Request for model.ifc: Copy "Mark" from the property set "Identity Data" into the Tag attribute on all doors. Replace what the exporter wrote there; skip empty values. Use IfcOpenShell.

First a look at what the model holds.

```python
import ifcopenshell
import ifcopenshell.util.element

model = ifcopenshell.open("model.ifc")
print(model.schema)
doors = model.by_type("IfcDoor")
print(len(doors), "doors")
for e in doors[:8]:
    source = ifcopenshell.util.element.get_pset(e, "Identity Data", "Mark")
    target = e.Tag
    print(e.id(), repr(source), repr(target), sep=" | ")
```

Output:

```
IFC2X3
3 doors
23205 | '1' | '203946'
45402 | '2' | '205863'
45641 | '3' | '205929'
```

```python
import ifcopenshell
import ifcopenshell.util.element

model = ifcopenshell.open("model.ifc")

count = 0
for e in model.by_type("IfcDoor"):
    value = ifcopenshell.util.element.get_pset(e, "Identity Data", "Mark")
    current = e.Tag
    if not value or not value.strip() or current == value:
        continue
    e.Tag = value
    count += 1

print(count, "doors updated")

model.write("model_v2.ifc")
```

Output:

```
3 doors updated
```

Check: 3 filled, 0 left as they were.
